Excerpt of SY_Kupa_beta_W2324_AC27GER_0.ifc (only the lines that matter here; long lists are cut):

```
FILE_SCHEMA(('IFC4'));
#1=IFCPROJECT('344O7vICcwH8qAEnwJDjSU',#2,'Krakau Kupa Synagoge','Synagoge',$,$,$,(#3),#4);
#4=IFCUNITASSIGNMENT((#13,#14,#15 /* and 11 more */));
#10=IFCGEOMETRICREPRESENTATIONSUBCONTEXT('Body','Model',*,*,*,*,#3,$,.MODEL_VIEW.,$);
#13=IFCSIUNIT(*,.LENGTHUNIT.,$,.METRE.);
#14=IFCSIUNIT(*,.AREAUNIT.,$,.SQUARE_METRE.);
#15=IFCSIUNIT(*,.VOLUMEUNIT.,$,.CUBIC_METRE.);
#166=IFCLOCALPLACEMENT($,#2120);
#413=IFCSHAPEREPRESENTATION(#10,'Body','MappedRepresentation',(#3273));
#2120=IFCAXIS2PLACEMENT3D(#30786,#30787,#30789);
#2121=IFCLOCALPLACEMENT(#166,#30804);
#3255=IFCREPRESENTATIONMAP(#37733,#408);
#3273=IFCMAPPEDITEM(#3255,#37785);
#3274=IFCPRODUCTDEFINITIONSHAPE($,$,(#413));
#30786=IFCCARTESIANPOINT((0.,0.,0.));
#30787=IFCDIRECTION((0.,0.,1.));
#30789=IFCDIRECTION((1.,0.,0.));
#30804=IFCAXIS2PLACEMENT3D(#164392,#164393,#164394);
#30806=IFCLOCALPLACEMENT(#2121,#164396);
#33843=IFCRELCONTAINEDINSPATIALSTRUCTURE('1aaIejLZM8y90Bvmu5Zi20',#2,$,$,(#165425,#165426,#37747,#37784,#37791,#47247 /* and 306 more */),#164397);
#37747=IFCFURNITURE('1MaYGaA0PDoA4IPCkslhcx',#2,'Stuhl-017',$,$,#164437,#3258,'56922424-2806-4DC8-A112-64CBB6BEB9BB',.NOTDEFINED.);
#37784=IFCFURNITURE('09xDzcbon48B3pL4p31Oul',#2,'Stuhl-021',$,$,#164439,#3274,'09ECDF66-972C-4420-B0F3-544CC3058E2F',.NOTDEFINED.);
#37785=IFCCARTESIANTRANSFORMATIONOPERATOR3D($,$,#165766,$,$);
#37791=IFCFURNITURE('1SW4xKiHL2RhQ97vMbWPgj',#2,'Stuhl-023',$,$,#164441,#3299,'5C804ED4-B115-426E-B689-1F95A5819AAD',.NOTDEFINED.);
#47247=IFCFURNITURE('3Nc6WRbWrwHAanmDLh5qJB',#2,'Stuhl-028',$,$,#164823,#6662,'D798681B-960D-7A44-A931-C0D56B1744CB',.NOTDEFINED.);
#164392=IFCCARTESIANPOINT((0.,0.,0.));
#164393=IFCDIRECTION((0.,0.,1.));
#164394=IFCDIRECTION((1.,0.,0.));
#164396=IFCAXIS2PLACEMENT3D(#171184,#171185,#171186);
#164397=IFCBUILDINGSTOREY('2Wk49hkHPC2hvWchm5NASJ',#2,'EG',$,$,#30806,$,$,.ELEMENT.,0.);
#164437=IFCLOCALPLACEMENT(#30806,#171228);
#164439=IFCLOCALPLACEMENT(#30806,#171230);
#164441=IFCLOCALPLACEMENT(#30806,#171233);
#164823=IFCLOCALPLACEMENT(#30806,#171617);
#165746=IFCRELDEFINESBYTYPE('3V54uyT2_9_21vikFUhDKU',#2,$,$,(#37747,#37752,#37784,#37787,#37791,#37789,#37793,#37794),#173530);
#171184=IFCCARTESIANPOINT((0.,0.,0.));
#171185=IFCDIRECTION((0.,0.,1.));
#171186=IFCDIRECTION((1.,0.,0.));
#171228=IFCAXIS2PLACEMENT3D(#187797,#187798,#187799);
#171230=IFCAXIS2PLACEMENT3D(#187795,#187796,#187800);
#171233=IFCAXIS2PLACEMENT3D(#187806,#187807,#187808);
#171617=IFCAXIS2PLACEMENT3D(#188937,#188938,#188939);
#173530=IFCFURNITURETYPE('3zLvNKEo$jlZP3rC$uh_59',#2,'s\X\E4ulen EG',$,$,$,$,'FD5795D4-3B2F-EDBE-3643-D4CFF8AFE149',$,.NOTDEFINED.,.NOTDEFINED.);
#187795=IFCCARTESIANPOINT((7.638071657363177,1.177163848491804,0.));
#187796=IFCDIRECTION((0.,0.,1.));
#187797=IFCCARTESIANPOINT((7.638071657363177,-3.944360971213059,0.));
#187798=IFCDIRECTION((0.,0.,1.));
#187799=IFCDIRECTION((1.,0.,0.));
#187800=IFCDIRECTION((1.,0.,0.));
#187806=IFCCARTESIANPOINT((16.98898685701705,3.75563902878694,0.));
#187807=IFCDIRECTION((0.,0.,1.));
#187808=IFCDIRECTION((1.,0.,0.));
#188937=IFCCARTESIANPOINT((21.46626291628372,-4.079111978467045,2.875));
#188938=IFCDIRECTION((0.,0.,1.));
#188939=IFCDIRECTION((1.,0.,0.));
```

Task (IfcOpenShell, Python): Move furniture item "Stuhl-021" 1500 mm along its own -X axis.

```python
import ifcopenshell
import ifcopenshell.api.geometry
import ifcopenshell.util.placement
import ifcopenshell.util.unit

model = ifcopenshell.open("SY_Kupa_beta_W2324_AC27GER_0.ifc")
unit_scale = ifcopenshell.util.unit.calculate_unit_scale(model)

item = model.by_guid("09xDzcbon48B3pL4p31Oul")
matrix = ifcopenshell.util.placement.get_local_placement(item.ObjectPlacement)
matrix[:3, 3] -= matrix[:3, 0] * 1.5 / unit_scale
ifcopenshell.api.geometry.edit_object_placement(model, product=item, matrix=matrix, is_si=False)

print(ifcopenshell.util.placement.get_local_placement(item.ObjectPlacement).round(3) + 0.0)

model.write("SY_Kupa_beta_W2324_AC27GER_0-out.ifc")
```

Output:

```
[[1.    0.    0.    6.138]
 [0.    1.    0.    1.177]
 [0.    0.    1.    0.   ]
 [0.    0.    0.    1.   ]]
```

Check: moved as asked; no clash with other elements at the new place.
